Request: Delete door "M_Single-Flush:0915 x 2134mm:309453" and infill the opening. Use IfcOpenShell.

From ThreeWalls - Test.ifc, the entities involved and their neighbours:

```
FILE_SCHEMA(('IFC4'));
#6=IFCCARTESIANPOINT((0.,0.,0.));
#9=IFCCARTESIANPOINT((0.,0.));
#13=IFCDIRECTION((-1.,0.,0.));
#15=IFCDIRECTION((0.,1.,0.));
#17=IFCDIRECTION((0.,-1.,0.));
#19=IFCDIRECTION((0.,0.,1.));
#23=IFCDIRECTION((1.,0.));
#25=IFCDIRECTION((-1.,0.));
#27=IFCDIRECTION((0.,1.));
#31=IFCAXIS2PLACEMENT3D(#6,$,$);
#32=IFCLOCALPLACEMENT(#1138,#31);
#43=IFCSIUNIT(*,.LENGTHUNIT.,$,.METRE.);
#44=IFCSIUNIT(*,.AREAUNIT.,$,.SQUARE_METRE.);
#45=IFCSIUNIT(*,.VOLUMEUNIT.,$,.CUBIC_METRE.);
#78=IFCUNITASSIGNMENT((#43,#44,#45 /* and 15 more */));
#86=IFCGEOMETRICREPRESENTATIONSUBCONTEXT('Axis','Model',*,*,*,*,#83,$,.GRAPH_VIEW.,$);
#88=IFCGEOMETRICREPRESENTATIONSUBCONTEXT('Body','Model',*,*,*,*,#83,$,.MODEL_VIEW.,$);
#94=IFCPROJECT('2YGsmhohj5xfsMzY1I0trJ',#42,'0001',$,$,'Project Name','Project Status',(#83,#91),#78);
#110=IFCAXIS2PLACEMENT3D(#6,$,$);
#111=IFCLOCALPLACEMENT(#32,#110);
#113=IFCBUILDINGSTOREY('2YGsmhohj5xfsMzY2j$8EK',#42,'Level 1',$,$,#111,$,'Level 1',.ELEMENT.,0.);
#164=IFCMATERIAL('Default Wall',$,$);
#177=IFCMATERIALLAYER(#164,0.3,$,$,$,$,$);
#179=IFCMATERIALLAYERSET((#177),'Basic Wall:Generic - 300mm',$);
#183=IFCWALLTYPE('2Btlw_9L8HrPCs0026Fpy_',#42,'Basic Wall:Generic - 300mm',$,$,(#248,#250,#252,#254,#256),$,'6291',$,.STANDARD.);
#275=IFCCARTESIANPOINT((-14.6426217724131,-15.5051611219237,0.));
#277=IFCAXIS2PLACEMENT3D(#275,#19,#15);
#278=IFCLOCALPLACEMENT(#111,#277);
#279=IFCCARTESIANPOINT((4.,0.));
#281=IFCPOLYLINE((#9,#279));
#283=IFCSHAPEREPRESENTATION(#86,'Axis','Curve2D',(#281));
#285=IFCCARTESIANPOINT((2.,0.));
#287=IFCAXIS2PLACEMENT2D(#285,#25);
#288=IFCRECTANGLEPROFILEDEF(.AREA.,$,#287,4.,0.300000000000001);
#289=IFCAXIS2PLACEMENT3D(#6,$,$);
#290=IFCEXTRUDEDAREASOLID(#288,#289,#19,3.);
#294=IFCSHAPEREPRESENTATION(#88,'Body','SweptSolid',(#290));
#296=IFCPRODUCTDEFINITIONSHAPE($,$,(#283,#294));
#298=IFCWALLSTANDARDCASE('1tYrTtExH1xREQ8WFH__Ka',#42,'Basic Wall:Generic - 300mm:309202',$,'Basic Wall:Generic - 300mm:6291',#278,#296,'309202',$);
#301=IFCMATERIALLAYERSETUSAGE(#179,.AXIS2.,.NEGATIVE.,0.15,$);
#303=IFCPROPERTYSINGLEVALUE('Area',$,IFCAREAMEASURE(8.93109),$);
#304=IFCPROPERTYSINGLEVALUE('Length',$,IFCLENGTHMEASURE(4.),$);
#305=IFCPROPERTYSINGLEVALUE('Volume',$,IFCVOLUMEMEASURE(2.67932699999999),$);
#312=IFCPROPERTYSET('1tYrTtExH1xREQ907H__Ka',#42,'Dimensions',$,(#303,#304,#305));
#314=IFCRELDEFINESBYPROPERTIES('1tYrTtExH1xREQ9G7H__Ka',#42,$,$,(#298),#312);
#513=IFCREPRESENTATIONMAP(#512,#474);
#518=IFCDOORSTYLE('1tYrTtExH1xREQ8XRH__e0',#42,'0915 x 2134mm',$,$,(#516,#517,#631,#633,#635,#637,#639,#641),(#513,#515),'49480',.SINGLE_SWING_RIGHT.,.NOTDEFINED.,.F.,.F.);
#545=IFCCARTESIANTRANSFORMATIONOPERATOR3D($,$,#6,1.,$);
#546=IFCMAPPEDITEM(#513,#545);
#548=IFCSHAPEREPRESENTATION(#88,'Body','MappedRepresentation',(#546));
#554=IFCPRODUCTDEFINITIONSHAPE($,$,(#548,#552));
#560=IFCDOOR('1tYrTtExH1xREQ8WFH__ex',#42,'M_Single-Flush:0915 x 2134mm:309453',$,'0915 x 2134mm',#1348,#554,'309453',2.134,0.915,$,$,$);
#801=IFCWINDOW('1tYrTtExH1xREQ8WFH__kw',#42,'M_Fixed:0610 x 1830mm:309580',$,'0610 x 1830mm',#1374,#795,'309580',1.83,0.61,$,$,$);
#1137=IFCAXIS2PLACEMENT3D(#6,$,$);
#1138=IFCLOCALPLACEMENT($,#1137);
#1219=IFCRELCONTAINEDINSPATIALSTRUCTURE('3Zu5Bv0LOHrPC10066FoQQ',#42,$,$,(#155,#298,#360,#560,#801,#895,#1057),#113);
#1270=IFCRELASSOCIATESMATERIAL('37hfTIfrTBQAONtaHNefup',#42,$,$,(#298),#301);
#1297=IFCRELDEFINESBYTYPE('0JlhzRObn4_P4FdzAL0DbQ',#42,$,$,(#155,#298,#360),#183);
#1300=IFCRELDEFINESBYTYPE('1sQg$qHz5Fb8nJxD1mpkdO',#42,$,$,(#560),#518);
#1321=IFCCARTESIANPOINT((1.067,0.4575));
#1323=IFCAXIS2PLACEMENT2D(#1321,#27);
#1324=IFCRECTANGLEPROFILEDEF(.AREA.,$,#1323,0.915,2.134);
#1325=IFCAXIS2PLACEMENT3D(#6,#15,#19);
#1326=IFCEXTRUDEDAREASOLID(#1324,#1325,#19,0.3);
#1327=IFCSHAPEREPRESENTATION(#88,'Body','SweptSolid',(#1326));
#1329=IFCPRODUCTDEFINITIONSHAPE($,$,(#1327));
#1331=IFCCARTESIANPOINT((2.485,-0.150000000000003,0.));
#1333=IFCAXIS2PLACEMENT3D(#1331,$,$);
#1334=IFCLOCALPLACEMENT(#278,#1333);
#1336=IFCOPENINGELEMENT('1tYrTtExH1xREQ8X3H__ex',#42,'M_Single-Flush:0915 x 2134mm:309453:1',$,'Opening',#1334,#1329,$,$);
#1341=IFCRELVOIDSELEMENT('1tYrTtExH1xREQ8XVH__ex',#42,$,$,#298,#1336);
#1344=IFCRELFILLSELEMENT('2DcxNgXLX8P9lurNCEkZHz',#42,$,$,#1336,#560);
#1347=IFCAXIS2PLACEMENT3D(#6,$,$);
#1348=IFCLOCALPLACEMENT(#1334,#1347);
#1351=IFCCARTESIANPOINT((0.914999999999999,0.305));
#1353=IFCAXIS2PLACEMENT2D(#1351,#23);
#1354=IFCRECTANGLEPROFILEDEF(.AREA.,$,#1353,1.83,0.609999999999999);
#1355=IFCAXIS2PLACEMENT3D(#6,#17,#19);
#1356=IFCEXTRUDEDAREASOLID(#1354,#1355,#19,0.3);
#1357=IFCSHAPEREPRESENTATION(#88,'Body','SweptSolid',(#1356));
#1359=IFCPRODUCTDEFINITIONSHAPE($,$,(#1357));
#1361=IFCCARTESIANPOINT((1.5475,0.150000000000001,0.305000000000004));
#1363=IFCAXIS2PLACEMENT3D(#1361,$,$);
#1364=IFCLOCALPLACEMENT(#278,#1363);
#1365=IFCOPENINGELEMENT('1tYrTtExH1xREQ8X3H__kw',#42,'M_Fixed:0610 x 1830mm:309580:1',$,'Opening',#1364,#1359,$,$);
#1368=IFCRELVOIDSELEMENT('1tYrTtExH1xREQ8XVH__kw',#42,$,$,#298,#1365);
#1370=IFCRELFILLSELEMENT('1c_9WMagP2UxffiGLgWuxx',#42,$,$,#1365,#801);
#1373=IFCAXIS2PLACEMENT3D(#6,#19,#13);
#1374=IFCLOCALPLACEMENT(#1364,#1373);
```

```python
import ifcopenshell
import ifcopenshell.api.feature
import ifcopenshell.api.pset
import ifcopenshell.api.root
import ifcopenshell.geom
import ifcopenshell.util.element
import ifcopenshell.util.shape
import ifcopenshell.util.unit

model = ifcopenshell.open("ThreeWalls - Test.ifc")
area_scale = ifcopenshell.util.unit.calculate_unit_scale(model, "AREAUNIT")
volume_scale = ifcopenshell.util.unit.calculate_unit_scale(model, "VOLUMEUNIT")
settings = ifcopenshell.geom.settings()


def volume(element):
    """Net volume in cubic metres, openings subtracted."""
    shape = ifcopenshell.geom.create_shape(settings, element)
    return ifcopenshell.util.shape.get_volume(shape.geometry)


door = model.by_id(560)
opening = door.FillsVoids[0].RelatingOpeningElement
wall = opening.VoidsElements[0].RelatingBuildingElement
before = volume(wall)

ifcopenshell.api.root.remove_product(model, product=door)
ifcopenshell.api.feature.remove_feature(model, feature=opening)

after = volume(wall)
thickness = 0.3  # wall thickness in metres

# Update the wall's stored quantities.
pset = model.by_id(ifcopenshell.util.element.get_pset(wall, "Dimensions", should_inherit=False)["id"])
ifcopenshell.api.pset.edit_pset(model, pset=pset, properties={
    "Area": model.create_entity("IfcAreaMeasure", after / thickness / area_scale),
    "Volume": model.create_entity("IfcVolumeMeasure", after / volume_scale),
})

print(f"wall volume {before:.3f} -> {after:.3f} m3")

model.write("ThreeWalls - Test_v2.ifc")
```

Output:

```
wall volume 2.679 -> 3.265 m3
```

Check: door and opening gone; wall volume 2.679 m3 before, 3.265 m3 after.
